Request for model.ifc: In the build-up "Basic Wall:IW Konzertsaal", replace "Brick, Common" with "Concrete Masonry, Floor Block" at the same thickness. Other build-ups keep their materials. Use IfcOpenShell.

First a look at what the model holds.

```python
import ifcopenshell
import ifcopenshell.util.element

model = ifcopenshell.open("model.ifc")
print(model.schema)
for layer_set in model.by_type("IfcMaterialLayerSet"):
    if layer_set.LayerSetName == "Basic Wall:IW Konzertsaal":
        for layer in layer_set.MaterialLayers:
            print(layer.id(), layer.Material and layer.Material.Name, layer.LayerThickness, sep=" | ")
        print(len(ifcopenshell.util.element.get_elements_by_material(model, layer_set)), "elements and types use it")
print(sorted(m.Name for m in model.by_type("IfcMaterial") if m.Name)[:60])
```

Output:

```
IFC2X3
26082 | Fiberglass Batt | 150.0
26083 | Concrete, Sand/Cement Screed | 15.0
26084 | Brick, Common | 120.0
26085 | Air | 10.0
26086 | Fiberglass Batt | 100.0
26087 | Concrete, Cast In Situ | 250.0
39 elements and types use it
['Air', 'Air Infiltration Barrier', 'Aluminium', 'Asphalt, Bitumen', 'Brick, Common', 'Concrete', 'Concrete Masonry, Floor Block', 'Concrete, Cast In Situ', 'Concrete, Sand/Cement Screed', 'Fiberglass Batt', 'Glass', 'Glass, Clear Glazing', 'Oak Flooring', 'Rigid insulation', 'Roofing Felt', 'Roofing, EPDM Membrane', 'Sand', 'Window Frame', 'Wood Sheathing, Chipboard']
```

```python
import ifcopenshell
import ifcopenshell.api.material

model = ifcopenshell.open("model.ifc")

layer_set = next(s for s in model.by_type("IfcMaterialLayerSet") if s.LayerSetName == "Basic Wall:IW Konzertsaal")
layer = next(l for l in layer_set.MaterialLayers if l.Material and l.Material.Name == "Brick, Common")
material = next(m for m in model.by_type("IfcMaterial") if m.Name == "Concrete Masonry, Floor Block")

# Point this one layer at the other material; renaming the old one would change it everywhere.
ifcopenshell.api.material.edit_layer(model, layer=layer, attributes={}, material=material)

print([l.Material.Name if l.Material else None for l in layer_set.MaterialLayers])

model.write("model-out.ifc")
```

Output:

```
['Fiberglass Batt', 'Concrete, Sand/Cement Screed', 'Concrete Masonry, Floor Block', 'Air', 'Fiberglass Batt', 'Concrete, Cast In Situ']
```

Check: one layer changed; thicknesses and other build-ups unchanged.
